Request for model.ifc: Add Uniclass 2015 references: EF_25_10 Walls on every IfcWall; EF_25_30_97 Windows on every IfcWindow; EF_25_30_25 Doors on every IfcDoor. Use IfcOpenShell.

First a look at what the model holds.

```python
import ifcopenshell

model = ifcopenshell.open("model.ifc")
print(model.schema)
print("classifications:", [c.Name for c in model.by_type("IfcClassification")])
for ifc_class in ("IfcDoor", "IfcRoof", "IfcStair", "IfcWall", "IfcWindow"):
    print(ifc_class, len(model.by_type(ifc_class)))
```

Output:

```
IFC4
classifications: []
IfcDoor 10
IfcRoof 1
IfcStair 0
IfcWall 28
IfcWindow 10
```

```python
import ifcopenshell
import ifcopenshell.api.classification

model = ifcopenshell.open("model.ifc")

system = ifcopenshell.api.classification.add_classification(model, classification="Uniclass 2015")

codes = {
    "IfcWall": ("EF_25_10", "Walls"),
    "IfcWindow": ("EF_25_30_97", "Windows"),
    "IfcDoor": ("EF_25_30_25", "Doors"),
}
for ifc_class, (code, name) in codes.items():
    products = model.by_type(ifc_class)
    ifcopenshell.api.classification.add_reference(
        model, products=products, classification=system, identification=code, name=name
    )
    print(code, len(products))

model.write("model_rev.ifc")
```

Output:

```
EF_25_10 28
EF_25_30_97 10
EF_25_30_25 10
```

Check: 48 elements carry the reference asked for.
